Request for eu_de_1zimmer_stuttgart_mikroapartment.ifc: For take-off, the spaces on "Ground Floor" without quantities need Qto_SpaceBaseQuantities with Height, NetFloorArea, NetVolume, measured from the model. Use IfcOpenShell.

First a look at what the model holds.

```python
import ifcopenshell
import ifcopenshell.util.element
import ifcopenshell.util.unit

model = ifcopenshell.open("eu_de_1zimmer_stuttgart_mikroapartment.ifc")
print(model.schema)
for unit_type in ("LENGTHUNIT", "AREAUNIT", "VOLUMEUNIT"):
    print(unit_type, ifcopenshell.util.unit.calculate_unit_scale(model, unit_type))
storey = next(s for s in model.by_type("IfcBuildingStorey") if s.Name == "Ground Floor")
spaces = [e for e in ifcopenshell.util.element.get_decomposition(storey) if e.is_a("IfcSpace")]
for e in sorted(spaces, key=lambda e: e.id()):
    print(e.id(), e.is_a(), e.Name, list(ifcopenshell.util.element.get_psets(e, qtos_only=True)), sep=" | ")
```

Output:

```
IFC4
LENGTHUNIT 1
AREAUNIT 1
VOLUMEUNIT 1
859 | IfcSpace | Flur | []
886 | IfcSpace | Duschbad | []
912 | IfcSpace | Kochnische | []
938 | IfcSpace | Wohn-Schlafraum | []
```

```python
import ifcopenshell
import ifcopenshell.api.pset
import ifcopenshell.geom
import ifcopenshell.util.element
import ifcopenshell.util.shape
import ifcopenshell.util.unit

model = ifcopenshell.open("eu_de_1zimmer_stuttgart_mikroapartment.ifc")
unit_scale = ifcopenshell.util.unit.calculate_unit_scale(model)
area_scale = ifcopenshell.util.unit.calculate_unit_scale(model, "AREAUNIT")
volume_scale = ifcopenshell.util.unit.calculate_unit_scale(model, "VOLUMEUNIT")
settings = ifcopenshell.geom.settings()

storey = next(s for s in model.by_type("IfcBuildingStorey") if s.Name == "Ground Floor")
spaces = [e for e in ifcopenshell.util.element.get_decomposition(storey) if e.is_a("IfcSpace")]

for e in sorted(spaces, key=lambda e: e.id()):
    if ifcopenshell.util.element.get_psets(e, qtos_only=True, should_inherit=False):
        continue
    # Geometry comes back in metres, in the element's own axes.
    shape = ifcopenshell.geom.create_shape(settings, e)
    values = {
        "Height": ifcopenshell.util.shape.get_z(shape.geometry) / unit_scale,
        "NetFloorArea": ifcopenshell.util.shape.get_footprint_area(shape.geometry) / area_scale,
        "NetVolume": ifcopenshell.util.shape.get_volume(shape.geometry) / volume_scale,
    }
    qto = ifcopenshell.api.pset.add_qto(model, product=e, name="Qto_SpaceBaseQuantities")
    ifcopenshell.api.pset.edit_qto(model, qto=qto, properties=values)
    print(e.id(), {k: round(v, 3) for k, v in values.items()})

model.write("eu_de_1zimmer_stuttgart_mikroapartment_v2.ifc")
```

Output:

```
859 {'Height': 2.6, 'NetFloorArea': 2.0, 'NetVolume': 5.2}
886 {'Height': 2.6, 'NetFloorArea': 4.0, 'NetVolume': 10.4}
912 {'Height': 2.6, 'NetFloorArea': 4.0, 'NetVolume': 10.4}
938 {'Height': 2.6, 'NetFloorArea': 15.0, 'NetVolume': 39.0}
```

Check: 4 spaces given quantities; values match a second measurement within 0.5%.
